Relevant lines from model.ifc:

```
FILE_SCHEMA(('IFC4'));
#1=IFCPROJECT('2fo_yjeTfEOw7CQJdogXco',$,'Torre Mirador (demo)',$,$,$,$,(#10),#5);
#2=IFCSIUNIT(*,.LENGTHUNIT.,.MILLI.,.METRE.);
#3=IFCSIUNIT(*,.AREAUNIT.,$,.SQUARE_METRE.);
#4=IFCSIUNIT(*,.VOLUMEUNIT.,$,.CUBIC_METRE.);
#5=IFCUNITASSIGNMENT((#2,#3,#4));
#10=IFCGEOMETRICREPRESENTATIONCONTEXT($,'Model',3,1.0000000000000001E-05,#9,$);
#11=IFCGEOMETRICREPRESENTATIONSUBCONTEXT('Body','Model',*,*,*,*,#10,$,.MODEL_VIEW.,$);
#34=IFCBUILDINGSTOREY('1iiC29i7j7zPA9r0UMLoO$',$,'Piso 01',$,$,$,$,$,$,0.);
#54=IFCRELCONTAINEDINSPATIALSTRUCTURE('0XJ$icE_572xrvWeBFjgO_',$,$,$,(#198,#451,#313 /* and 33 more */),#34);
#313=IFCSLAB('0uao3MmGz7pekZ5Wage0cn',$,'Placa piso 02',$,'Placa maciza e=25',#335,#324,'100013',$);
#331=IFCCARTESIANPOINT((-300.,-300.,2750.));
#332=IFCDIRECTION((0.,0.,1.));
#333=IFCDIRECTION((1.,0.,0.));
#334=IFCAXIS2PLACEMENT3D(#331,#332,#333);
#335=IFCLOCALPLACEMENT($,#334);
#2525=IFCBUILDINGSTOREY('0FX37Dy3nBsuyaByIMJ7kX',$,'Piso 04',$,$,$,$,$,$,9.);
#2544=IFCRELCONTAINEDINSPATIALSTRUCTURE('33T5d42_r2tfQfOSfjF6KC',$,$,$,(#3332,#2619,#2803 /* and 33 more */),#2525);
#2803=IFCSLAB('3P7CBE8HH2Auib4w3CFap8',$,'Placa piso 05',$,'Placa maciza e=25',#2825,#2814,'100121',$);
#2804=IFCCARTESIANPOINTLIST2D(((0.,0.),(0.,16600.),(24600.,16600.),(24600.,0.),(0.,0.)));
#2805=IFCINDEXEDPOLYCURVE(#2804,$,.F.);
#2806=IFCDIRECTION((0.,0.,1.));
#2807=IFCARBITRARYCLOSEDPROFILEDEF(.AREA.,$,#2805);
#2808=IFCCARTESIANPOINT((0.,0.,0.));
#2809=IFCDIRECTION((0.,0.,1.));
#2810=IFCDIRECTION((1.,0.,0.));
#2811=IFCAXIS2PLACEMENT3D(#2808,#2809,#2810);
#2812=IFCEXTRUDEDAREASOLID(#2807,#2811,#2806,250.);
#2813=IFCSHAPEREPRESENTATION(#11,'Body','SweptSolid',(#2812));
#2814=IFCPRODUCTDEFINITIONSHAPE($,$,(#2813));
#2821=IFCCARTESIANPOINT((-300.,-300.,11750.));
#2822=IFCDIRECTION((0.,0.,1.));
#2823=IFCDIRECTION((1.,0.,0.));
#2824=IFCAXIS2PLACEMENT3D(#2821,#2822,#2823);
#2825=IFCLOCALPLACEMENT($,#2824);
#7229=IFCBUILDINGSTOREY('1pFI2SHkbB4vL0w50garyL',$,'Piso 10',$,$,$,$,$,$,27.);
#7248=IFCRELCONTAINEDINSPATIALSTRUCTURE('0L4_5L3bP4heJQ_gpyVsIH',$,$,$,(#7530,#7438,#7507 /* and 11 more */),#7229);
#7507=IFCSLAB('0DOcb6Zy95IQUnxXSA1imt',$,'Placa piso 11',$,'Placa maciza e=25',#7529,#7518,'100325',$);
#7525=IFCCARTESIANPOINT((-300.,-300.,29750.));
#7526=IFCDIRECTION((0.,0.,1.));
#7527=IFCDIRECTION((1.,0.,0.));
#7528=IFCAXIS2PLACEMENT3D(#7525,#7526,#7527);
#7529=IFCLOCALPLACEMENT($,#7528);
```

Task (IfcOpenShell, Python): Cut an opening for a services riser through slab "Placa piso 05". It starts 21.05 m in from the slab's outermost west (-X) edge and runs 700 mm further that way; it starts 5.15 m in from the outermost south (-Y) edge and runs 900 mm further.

```python
import numpy as np
import ifcopenshell
import ifcopenshell.api.feature
import ifcopenshell.api.geometry
import ifcopenshell.api.root
import ifcopenshell.geom
import ifcopenshell.util.placement
import ifcopenshell.util.representation
import ifcopenshell.util.shape
import ifcopenshell.util.unit

model = ifcopenshell.open("model.ifc")
unit_scale = ifcopenshell.util.unit.calculate_unit_scale(model)
settings = ifcopenshell.geom.settings()


def volume(element):
    """Net volume in cubic metres, openings subtracted."""
    shape = ifcopenshell.geom.create_shape(settings, element)
    return ifcopenshell.util.shape.get_volume(shape.geometry)


slab = model.by_id(2803)
before = volume(slab)

# Extent in the slab's own axes, in metres. The edges named are its -X and -Y sides.
slab_shape = ifcopenshell.geom.create_shape(settings, slab)
vertices = ifcopenshell.util.shape.get_vertices(slab_shape.geometry)
x_min, y_min, bottom = vertices.min(axis=0)
top = vertices[:, 2].max()

opening = ifcopenshell.api.root.create_entity(model, ifc_class="IfcOpeningElement", name="Services riser opening", predefined_type="OPENING")
context = ifcopenshell.util.representation.get_context(model, "Model", "Body", "MODEL_VIEW")
width, depth = 0.7, 0.9
outline = [(0.0, 0.0), (width, 0.0), (width, depth), (0.0, depth), (0.0, 0.0)]
# Overshoot both faces by 50 mm so the cut is clean.
shape = ifcopenshell.api.geometry.add_slab_representation(
    model, context=context, depth=top - bottom + 0.1, polyline=outline
)
ifcopenshell.api.geometry.assign_representation(model, product=opening, representation=shape)

matrix = ifcopenshell.util.placement.get_local_placement(slab.ObjectPlacement)
matrix[:, 3] = matrix @ np.append(np.array([x_min + 21.05, y_min + 5.15, bottom - 0.05]) / unit_scale, 1.0)
ifcopenshell.api.geometry.edit_object_placement(model, product=opening, matrix=matrix, is_si=False)
ifcopenshell.api.feature.add_feature(model, feature=opening, element=slab)

after = volume(slab)

print(f"slab volume {before:.3f} -> {after:.3f} m3")

model.write("model_v2.ifc")
```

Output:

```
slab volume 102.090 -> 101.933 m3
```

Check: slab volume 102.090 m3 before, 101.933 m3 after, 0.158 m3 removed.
